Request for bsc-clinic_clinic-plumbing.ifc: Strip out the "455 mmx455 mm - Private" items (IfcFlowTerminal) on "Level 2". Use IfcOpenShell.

First a look at what the model holds.

```python
import ifcopenshell
import ifcopenshell.util.element

model = ifcopenshell.open("bsc-clinic_clinic-plumbing.ifc")
print(model.schema)
storey = next(s for s in model.by_type("IfcBuildingStorey") if s.Name == "Level 2")
terminals = [e for e in ifcopenshell.util.element.get_decomposition(storey) if e.is_a("IfcFlowTerminal")]
seen = {}
for e in terminals:
    element_type = ifcopenshell.util.element.get_type(e)
    name = element_type.Name if element_type not in (None, e) else None
    seen[name] = seen.get(name, 0) + 1
for name, count in sorted(seen.items(), key=str):
    print(count, "x", name)
```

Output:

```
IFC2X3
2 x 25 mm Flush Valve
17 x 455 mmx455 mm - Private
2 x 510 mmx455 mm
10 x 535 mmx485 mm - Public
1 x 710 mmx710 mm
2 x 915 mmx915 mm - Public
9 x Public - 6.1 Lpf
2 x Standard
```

```python
import ifcopenshell
import ifcopenshell.api.root
import ifcopenshell.util.element

model = ifcopenshell.open("bsc-clinic_clinic-plumbing.ifc")

storey = next(s for s in model.by_type("IfcBuildingStorey") if s.Name == "Level 2")
terminals = [e for e in ifcopenshell.util.element.get_decomposition(storey) if e.is_a("IfcFlowTerminal")]
targets = [e for e in terminals if (t := ifcopenshell.util.element.get_type(e)) not in (None, e) and t.Name == "455 mmx455 mm - Private"]

for e in targets:
    ifcopenshell.api.root.remove_product(model, product=e)
print(len(targets), "removed")

model.write("bsc-clinic_clinic-plumbing_updated.ifc")
```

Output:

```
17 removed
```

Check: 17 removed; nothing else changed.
